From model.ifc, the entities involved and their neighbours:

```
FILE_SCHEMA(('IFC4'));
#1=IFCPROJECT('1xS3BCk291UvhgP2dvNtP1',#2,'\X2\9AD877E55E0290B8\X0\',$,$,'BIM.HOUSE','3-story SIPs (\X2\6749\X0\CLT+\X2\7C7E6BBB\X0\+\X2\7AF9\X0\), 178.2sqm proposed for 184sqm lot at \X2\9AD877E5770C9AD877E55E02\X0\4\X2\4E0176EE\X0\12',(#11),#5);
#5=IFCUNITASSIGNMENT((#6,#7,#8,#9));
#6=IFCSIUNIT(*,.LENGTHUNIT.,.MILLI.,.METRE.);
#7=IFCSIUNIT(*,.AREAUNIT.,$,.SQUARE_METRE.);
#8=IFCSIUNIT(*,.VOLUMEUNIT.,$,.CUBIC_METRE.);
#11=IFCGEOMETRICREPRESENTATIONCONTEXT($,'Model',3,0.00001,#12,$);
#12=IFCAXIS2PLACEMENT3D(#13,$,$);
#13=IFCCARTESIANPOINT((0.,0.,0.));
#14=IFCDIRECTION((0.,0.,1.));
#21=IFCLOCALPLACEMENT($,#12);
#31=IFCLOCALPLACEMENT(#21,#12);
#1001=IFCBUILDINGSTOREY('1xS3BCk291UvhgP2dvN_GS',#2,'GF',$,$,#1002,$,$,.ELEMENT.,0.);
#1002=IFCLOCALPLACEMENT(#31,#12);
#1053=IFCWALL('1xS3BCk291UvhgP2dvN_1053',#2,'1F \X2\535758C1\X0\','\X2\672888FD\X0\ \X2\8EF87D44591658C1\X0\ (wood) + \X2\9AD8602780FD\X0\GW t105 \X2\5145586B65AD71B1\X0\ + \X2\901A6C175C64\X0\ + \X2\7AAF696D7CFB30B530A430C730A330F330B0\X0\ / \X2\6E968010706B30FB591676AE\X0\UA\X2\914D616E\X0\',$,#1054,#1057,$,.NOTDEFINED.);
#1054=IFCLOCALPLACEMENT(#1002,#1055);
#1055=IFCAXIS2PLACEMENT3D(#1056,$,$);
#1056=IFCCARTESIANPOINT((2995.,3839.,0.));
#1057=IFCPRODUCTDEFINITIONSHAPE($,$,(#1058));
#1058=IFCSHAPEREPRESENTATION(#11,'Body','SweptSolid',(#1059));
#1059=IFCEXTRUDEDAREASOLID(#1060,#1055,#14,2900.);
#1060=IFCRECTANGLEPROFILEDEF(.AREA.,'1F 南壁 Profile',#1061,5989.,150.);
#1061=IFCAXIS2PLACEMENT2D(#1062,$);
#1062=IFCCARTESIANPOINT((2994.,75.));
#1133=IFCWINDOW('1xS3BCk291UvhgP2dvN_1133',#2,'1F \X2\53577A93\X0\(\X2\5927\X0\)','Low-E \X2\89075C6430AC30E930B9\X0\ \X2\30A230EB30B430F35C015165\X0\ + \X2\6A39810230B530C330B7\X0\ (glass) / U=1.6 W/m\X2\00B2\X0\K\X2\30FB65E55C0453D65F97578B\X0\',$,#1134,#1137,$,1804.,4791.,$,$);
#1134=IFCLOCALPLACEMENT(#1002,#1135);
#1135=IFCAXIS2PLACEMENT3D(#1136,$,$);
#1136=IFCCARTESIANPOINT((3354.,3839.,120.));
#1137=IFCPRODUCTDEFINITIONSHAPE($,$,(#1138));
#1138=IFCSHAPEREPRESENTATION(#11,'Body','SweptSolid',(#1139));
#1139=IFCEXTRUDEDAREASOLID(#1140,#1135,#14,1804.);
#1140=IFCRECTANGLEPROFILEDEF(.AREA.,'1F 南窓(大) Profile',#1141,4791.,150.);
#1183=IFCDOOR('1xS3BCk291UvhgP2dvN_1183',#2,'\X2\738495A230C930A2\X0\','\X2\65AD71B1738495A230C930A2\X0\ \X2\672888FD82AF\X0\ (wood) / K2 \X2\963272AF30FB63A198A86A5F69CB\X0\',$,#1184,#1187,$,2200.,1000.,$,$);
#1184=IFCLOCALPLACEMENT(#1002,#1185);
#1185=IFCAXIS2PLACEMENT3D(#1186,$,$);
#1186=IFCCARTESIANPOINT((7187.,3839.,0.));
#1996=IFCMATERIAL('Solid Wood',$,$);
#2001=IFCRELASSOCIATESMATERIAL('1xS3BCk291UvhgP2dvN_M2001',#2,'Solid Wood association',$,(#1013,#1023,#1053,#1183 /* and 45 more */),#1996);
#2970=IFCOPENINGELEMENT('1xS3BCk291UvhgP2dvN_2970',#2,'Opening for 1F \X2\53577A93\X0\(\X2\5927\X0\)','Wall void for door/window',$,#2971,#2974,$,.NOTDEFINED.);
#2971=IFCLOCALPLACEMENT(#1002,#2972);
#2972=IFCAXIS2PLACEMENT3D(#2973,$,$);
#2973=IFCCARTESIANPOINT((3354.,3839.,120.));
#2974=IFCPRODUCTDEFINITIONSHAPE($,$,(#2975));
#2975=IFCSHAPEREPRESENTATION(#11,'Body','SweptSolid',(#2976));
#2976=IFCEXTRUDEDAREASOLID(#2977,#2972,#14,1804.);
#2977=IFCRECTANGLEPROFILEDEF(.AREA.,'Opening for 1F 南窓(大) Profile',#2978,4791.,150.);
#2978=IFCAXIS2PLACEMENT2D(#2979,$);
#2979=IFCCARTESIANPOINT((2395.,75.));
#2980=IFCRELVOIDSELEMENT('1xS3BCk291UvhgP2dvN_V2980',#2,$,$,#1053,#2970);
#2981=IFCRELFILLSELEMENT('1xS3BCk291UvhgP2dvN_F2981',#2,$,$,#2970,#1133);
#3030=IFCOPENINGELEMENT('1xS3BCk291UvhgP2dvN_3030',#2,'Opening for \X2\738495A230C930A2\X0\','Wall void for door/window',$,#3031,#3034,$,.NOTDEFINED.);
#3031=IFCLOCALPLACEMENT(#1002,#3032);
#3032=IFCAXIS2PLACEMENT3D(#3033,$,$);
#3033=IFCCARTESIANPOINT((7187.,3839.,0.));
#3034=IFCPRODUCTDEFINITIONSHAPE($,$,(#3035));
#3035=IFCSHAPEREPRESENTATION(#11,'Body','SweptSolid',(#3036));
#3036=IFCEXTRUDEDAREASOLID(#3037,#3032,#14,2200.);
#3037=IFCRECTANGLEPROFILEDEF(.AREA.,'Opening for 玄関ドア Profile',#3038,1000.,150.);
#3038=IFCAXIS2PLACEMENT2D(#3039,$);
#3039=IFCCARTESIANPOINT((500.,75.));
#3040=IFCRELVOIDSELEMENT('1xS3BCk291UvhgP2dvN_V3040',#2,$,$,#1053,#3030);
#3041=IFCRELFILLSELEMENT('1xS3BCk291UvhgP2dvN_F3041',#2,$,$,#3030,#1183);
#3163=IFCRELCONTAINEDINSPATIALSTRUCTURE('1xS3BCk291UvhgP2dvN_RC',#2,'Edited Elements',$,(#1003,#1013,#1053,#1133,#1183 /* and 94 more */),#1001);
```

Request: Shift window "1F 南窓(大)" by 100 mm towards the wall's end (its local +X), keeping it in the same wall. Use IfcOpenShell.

```python
import ifcopenshell
import ifcopenshell.api.geometry
import ifcopenshell.util.placement
import ifcopenshell.util.unit

model = ifcopenshell.open("model.ifc")
unit_scale = ifcopenshell.util.unit.calculate_unit_scale(model)

window = model.by_guid("1xS3BCk291UvhgP2dvN_1133")
opening = window.FillsVoids[0].RelatingOpeningElement
wall = opening.VoidsElements[0].RelatingBuildingElement

wall_matrix = ifcopenshell.util.placement.get_local_placement(wall.ObjectPlacement)
shift = wall_matrix[:3, 0] * 0.1 / unit_scale
before = ifcopenshell.util.placement.get_local_placement(window.ObjectPlacement)[:3, 3].copy()

# The window is not placed relative to its opening, so move both.
for product in (opening, window):
    matrix = ifcopenshell.util.placement.get_local_placement(product.ObjectPlacement)
    matrix[:3, 3] += shift
    ifcopenshell.api.geometry.edit_object_placement(model, product=product, matrix=matrix, is_si=False)

after = ifcopenshell.util.placement.get_local_placement(window.ObjectPlacement)[:3, 3]
print("window moved by", (after - before).round(3) + 0.0)

model.write("model_rev.ifc")
```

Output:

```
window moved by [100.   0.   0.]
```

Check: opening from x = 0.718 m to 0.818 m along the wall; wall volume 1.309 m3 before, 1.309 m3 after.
